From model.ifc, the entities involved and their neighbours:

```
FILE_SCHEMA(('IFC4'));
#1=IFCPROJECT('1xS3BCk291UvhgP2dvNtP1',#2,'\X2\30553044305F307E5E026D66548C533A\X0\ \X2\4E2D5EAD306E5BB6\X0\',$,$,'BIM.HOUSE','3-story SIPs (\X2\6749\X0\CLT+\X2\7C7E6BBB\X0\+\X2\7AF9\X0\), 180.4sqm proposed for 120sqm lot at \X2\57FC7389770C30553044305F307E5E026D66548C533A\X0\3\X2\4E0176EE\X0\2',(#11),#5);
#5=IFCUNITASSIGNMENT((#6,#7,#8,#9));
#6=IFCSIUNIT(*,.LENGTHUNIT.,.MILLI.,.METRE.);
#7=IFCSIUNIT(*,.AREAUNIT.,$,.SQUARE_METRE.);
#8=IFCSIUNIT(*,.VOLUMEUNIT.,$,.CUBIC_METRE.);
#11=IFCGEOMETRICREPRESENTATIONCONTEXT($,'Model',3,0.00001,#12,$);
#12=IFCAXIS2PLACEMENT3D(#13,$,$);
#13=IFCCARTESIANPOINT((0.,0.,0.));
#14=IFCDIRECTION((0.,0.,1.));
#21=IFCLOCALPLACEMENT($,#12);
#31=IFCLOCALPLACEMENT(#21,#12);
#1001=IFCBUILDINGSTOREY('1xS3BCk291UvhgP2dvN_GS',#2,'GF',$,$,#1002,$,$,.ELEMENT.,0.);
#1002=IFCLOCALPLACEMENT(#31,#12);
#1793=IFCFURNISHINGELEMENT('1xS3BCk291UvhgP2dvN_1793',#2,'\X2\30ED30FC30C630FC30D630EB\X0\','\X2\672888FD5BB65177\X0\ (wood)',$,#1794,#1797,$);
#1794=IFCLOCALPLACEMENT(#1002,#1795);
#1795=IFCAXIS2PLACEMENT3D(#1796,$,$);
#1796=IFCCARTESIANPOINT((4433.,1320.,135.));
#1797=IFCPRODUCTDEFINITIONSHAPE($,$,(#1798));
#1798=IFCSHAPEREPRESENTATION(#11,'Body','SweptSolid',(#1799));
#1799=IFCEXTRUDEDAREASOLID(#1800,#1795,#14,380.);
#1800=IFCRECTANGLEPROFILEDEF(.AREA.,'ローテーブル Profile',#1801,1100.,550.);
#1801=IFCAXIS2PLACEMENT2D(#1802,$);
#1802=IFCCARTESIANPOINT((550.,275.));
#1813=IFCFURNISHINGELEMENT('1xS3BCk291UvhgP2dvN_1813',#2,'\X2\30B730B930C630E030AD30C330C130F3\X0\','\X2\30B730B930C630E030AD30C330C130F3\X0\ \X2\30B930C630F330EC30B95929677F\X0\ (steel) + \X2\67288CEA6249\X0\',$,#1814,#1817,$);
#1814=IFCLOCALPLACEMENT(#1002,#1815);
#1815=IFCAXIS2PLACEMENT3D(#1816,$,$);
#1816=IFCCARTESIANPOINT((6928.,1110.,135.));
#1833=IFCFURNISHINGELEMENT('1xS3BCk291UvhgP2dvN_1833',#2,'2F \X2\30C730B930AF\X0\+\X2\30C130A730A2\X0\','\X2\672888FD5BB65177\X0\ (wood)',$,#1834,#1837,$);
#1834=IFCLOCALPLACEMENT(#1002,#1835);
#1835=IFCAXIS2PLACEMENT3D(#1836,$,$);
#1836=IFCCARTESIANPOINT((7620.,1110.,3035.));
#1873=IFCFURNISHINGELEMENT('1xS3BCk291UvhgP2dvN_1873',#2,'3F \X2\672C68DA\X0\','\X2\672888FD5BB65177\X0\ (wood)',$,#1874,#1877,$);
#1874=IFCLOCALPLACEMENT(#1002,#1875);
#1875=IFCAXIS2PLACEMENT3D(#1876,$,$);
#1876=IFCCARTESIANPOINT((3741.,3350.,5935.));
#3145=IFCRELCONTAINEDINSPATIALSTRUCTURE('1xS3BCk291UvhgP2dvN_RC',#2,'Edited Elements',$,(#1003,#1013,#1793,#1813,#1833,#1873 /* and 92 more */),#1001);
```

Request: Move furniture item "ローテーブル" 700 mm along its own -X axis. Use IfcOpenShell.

```python
import ifcopenshell
import ifcopenshell.api.geometry
import ifcopenshell.util.placement
import ifcopenshell.util.unit

model = ifcopenshell.open("model.ifc")
unit_scale = ifcopenshell.util.unit.calculate_unit_scale(model)

item = model.by_guid("1xS3BCk291UvhgP2dvN_1793")
matrix = ifcopenshell.util.placement.get_local_placement(item.ObjectPlacement)
matrix[:3, 3] -= matrix[:3, 0] * 0.7 / unit_scale
ifcopenshell.api.geometry.edit_object_placement(model, product=item, matrix=matrix, is_si=False)

print(ifcopenshell.util.placement.get_local_placement(item.ObjectPlacement).round(3) + 0.0)

model.write("model_edited.ifc")
```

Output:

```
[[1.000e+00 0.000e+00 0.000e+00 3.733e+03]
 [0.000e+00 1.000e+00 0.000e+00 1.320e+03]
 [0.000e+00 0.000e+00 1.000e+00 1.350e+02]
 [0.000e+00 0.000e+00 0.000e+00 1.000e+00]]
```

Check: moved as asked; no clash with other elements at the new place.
